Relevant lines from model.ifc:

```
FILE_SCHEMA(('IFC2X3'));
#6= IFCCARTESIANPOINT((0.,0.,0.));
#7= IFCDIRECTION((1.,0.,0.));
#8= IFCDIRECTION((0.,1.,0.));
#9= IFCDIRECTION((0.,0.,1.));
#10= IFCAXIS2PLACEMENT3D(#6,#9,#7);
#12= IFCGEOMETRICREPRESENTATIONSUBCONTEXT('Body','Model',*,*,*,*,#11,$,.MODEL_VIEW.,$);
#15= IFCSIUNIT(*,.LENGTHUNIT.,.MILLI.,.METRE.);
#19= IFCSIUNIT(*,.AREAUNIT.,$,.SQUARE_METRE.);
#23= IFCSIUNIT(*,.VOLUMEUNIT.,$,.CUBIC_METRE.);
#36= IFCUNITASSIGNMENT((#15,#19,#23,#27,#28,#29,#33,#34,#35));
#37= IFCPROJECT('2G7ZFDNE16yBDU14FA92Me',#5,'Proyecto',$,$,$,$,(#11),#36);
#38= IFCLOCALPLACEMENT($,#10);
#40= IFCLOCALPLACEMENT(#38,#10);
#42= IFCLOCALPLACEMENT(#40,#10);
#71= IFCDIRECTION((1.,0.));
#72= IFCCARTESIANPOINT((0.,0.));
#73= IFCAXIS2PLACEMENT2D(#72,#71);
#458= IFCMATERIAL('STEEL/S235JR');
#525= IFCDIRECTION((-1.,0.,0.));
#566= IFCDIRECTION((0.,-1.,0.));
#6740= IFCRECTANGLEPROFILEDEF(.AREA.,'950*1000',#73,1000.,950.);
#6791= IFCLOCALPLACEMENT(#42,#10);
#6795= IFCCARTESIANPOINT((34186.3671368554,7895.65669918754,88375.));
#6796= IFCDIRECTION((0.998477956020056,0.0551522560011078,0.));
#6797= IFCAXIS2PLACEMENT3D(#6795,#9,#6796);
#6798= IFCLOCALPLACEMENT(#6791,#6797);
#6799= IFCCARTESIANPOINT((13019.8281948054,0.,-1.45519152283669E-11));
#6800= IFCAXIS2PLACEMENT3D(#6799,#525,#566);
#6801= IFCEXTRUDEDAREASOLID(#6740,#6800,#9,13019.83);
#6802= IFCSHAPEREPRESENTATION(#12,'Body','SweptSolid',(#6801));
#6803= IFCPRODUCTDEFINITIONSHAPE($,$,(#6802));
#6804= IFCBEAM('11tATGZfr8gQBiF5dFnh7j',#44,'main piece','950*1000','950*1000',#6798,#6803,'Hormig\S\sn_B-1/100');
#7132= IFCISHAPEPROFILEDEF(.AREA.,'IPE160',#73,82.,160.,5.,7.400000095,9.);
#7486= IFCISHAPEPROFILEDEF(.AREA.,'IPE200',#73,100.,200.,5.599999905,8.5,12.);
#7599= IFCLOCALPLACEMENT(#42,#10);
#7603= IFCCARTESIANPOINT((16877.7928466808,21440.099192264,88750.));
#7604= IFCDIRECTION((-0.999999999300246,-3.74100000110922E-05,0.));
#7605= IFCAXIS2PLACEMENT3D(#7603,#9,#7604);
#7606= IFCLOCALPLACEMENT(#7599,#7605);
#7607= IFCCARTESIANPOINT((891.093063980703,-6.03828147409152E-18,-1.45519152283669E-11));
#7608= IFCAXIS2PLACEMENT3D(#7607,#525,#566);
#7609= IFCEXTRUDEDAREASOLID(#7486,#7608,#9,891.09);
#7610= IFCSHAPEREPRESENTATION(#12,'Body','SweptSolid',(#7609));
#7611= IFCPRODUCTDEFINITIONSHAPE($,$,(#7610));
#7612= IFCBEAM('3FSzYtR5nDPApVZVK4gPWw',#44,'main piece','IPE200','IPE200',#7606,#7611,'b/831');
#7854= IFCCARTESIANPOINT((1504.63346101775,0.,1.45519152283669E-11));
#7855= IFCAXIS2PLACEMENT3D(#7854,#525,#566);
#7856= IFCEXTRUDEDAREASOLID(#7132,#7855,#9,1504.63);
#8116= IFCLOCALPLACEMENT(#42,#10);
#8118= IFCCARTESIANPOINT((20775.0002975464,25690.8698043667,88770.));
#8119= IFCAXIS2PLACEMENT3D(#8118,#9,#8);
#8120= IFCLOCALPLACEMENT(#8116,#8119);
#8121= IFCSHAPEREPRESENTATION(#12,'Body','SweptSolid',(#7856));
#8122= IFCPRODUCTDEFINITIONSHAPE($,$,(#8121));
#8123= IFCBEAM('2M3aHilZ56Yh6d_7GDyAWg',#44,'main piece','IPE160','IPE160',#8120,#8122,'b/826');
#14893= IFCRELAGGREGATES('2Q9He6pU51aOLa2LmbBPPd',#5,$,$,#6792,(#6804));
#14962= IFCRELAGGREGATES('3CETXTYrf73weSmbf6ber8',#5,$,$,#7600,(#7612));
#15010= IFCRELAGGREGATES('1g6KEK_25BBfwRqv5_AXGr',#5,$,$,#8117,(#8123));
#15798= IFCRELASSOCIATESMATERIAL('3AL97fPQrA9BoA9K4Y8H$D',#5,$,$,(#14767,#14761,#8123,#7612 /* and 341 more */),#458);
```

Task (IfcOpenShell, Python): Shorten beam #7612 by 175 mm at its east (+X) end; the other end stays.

```python
import ifcopenshell
import ifcopenshell.util.representation
import ifcopenshell.util.unit

model = ifcopenshell.open("model.ifc")
unit_scale = ifcopenshell.util.unit.calculate_unit_scale(model)

member = model.by_guid("3FSzYtR5nDPApVZVK4gPWw")
change = -0.175 / unit_scale

# The extrusion runs towards the end named, so only its depth changes.
body = ifcopenshell.util.representation.get_representation(member, "Model", "Body")
solid = body.Items[0]
old_length = solid.Depth
solid.Depth += change

print(f"length {old_length:g} -> {solid.Depth:g}")

model.write("model_edited.ifc")
```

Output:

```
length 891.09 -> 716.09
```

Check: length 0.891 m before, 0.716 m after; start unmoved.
